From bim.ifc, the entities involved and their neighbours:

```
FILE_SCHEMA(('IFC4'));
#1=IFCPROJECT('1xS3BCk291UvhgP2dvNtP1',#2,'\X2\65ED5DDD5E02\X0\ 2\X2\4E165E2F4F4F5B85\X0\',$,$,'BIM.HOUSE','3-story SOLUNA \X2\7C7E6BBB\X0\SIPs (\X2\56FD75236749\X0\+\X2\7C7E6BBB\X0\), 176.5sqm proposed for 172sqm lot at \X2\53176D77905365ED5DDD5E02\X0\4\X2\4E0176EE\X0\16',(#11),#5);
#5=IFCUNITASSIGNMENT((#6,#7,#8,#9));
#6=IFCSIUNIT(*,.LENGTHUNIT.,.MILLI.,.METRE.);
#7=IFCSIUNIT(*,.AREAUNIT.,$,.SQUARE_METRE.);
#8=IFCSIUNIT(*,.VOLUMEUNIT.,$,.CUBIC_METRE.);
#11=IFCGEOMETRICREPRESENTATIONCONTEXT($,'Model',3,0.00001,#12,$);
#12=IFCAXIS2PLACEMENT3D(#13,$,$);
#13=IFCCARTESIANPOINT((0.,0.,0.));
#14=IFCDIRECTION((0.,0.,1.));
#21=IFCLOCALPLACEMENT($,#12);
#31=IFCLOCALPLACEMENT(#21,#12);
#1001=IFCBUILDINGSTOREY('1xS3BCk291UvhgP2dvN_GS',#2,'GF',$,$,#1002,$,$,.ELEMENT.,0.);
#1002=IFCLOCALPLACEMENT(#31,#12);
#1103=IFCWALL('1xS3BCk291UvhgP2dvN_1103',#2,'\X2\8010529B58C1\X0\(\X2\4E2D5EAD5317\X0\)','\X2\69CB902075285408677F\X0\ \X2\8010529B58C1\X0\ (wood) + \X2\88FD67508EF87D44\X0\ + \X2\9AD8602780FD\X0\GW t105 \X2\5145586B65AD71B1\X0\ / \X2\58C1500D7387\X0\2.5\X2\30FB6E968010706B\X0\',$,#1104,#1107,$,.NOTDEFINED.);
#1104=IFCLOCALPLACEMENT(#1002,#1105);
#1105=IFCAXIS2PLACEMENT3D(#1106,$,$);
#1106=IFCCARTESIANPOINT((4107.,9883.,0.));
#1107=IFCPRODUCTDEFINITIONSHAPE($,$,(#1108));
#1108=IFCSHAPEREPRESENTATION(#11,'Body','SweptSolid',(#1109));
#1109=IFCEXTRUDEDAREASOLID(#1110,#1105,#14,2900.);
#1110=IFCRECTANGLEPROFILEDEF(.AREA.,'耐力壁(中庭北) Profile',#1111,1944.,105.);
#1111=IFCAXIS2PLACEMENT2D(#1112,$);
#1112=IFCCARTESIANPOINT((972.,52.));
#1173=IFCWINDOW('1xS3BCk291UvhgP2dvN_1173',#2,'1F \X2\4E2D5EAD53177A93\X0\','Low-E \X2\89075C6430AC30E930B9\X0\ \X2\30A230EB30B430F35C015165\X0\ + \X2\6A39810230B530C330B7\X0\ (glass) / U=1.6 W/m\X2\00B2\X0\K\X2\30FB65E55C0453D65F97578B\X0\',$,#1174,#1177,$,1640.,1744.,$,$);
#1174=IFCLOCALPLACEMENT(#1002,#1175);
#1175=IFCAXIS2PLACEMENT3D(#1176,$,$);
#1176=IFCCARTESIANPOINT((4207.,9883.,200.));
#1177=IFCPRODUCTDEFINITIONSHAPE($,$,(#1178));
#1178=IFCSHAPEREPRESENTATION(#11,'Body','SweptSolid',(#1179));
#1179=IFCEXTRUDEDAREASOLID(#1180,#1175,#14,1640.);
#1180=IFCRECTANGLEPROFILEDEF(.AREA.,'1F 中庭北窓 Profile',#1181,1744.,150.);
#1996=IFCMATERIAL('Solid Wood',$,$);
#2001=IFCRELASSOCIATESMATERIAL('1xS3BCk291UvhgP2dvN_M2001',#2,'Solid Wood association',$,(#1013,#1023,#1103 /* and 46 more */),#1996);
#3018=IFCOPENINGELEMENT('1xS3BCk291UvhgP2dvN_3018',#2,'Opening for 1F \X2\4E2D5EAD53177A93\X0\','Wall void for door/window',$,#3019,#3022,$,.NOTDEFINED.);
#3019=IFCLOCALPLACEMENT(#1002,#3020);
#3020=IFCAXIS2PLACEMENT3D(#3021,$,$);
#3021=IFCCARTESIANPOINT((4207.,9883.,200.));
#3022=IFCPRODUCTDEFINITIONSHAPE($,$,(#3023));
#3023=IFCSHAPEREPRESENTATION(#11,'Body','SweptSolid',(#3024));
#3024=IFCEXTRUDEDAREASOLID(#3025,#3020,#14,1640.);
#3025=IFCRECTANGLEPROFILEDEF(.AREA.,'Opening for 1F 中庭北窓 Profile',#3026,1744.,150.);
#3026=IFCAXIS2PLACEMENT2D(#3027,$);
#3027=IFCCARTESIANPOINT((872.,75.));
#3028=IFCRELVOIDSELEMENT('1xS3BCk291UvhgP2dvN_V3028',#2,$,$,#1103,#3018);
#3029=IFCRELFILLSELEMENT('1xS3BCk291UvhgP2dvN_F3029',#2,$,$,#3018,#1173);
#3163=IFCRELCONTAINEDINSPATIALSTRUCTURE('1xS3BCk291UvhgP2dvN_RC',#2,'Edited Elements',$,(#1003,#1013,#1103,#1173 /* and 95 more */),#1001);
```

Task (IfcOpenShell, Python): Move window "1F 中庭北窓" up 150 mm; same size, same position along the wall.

```python
import numpy as np
import ifcopenshell
import ifcopenshell.api.geometry
import ifcopenshell.util.placement
import ifcopenshell.util.unit

model = ifcopenshell.open("bim.ifc")
unit_scale = ifcopenshell.util.unit.calculate_unit_scale(model)

window = model.by_guid("1xS3BCk291UvhgP2dvN_1173")
opening = window.FillsVoids[0].RelatingOpeningElement
dz = 150.0

shift = np.array([0.0, 0.0, dz])
# The window is not placed relative to its opening, so move both.
for product in (opening, window):
    matrix = ifcopenshell.util.placement.get_local_placement(product.ObjectPlacement)
    matrix[:3, 3] += shift
    ifcopenshell.api.geometry.edit_object_placement(model, product=product, matrix=matrix, is_si=False)

print(f"moved by {dz * unit_scale:+.3f} m")

model.write("bim_updated.ifc")
```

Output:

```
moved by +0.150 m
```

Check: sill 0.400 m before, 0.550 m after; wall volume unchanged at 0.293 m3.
